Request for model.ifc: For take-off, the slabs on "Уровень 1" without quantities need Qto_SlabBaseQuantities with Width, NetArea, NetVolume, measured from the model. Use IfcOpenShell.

First a look at what the model holds.

```python
import ifcopenshell
import ifcopenshell.util.element
import ifcopenshell.util.unit

model = ifcopenshell.open("model.ifc")
print(model.schema)
for unit_type in ("LENGTHUNIT", "AREAUNIT", "VOLUMEUNIT"):
    print(unit_type, ifcopenshell.util.unit.calculate_unit_scale(model, unit_type))
storey = next(s for s in model.by_type("IfcBuildingStorey") if s.Name == "Уровень 1")
slabs = [e for e in ifcopenshell.util.element.get_decomposition(storey) if e.is_a("IfcSlab")]
for e in sorted(slabs, key=lambda e: e.id()):
    print(e.id(), e.is_a(), e.Name, list(ifcopenshell.util.element.get_psets(e, qtos_only=True)), sep=" | ")
```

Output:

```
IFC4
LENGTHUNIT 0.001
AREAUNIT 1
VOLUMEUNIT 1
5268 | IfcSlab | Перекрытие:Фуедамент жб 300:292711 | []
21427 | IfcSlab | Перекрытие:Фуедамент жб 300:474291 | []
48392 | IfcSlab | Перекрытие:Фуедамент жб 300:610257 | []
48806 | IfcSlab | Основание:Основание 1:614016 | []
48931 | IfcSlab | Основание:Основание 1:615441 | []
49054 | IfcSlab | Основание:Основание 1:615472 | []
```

```python
import ifcopenshell
import ifcopenshell.api.pset
import ifcopenshell.geom
import ifcopenshell.util.element
import ifcopenshell.util.shape
import ifcopenshell.util.unit

model = ifcopenshell.open("model.ifc")
unit_scale = ifcopenshell.util.unit.calculate_unit_scale(model)
area_scale = ifcopenshell.util.unit.calculate_unit_scale(model, "AREAUNIT")
volume_scale = ifcopenshell.util.unit.calculate_unit_scale(model, "VOLUMEUNIT")
settings = ifcopenshell.geom.settings()

storey = next(s for s in model.by_type("IfcBuildingStorey") if s.Name == "Уровень 1")
slabs = [e for e in ifcopenshell.util.element.get_decomposition(storey) if e.is_a("IfcSlab")]

for e in sorted(slabs, key=lambda e: e.id()):
    if ifcopenshell.util.element.get_psets(e, qtos_only=True, should_inherit=False):
        continue
    # Geometry comes back in metres, in the element's own axes.
    shape = ifcopenshell.geom.create_shape(settings, e)
    values = {
        "Width": ifcopenshell.util.shape.get_z(shape.geometry) / unit_scale,
        "NetArea": ifcopenshell.util.shape.get_footprint_area(shape.geometry) / area_scale,
        "NetVolume": ifcopenshell.util.shape.get_volume(shape.geometry) / volume_scale,
    }
    qto = ifcopenshell.api.pset.add_qto(model, product=e, name="Qto_SlabBaseQuantities")
    ifcopenshell.api.pset.edit_qto(model, qto=qto, properties=values)
    print(e.id(), {k: round(v, 3) for k, v in values.items()})

model.write("model_rev.ifc")
```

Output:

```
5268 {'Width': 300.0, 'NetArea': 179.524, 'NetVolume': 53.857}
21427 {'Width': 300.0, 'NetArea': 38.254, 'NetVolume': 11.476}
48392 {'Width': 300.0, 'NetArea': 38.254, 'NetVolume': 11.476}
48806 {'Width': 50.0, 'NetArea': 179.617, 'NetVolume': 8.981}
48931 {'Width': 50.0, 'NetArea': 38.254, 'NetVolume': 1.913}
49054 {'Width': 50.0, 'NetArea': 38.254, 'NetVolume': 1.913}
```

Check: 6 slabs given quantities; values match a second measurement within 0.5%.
